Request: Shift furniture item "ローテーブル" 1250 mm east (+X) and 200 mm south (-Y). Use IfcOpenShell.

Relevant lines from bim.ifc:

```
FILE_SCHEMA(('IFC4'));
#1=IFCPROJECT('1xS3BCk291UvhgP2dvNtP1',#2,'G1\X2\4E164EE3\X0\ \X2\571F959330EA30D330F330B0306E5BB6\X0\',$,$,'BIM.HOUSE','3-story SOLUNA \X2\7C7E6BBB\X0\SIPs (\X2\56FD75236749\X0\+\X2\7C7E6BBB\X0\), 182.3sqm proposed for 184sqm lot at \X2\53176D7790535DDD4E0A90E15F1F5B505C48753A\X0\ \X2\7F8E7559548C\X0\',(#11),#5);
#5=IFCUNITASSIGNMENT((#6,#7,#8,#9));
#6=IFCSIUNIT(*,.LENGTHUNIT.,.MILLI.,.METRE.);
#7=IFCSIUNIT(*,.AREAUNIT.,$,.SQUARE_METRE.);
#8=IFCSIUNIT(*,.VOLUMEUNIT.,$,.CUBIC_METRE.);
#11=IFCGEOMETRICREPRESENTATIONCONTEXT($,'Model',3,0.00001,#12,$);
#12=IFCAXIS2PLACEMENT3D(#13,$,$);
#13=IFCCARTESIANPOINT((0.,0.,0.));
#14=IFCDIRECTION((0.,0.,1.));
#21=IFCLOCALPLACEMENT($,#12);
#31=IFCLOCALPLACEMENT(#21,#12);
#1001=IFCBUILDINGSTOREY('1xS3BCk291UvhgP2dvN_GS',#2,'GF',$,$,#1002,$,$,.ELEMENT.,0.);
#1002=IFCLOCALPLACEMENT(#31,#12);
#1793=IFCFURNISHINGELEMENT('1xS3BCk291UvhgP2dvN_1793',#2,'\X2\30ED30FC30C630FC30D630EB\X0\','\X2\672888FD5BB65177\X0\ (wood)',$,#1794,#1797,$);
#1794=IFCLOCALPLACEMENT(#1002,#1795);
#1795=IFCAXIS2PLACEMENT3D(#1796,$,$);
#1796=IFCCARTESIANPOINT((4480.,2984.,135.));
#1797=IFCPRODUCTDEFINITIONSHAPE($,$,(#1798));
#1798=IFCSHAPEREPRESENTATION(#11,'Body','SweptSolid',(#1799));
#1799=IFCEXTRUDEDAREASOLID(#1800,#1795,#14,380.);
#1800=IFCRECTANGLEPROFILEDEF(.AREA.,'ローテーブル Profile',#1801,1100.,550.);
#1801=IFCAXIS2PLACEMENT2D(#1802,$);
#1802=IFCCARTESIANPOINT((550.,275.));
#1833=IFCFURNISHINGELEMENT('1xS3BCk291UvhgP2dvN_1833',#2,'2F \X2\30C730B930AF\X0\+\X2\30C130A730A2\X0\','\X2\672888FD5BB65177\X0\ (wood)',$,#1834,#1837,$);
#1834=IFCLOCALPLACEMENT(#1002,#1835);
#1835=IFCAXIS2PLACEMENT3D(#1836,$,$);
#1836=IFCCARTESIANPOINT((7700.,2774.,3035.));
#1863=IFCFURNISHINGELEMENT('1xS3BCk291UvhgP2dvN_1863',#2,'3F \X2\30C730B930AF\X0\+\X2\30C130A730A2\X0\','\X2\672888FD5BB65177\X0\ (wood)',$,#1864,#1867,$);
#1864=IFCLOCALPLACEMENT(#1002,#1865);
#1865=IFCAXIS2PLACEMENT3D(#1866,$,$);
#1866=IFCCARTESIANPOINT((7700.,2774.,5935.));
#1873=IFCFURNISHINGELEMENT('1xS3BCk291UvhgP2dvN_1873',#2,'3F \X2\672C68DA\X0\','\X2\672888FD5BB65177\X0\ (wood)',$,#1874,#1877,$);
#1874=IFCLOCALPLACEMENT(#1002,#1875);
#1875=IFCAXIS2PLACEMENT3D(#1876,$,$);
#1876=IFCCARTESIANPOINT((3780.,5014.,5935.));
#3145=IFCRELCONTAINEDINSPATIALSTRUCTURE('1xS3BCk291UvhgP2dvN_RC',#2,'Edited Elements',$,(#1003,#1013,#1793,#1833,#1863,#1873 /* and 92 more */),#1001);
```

```python
import ifcopenshell
import ifcopenshell.api.geometry
import ifcopenshell.util.placement
import ifcopenshell.util.unit

model = ifcopenshell.open("bim.ifc")
unit_scale = ifcopenshell.util.unit.calculate_unit_scale(model)

item = model.by_guid("1xS3BCk291UvhgP2dvN_1793")
matrix = ifcopenshell.util.placement.get_local_placement(item.ObjectPlacement)
matrix[0, 3] += 1.25 / unit_scale
matrix[1, 3] -= 0.2 / unit_scale
ifcopenshell.api.geometry.edit_object_placement(model, product=item, matrix=matrix, is_si=False)

print(ifcopenshell.util.placement.get_local_placement(item.ObjectPlacement).round(3) + 0.0)

model.write("bim_edited.ifc")
```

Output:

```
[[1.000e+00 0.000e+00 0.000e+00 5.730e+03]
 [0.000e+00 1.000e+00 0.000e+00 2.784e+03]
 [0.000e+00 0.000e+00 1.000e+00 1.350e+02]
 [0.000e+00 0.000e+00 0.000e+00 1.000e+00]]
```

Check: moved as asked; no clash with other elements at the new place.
